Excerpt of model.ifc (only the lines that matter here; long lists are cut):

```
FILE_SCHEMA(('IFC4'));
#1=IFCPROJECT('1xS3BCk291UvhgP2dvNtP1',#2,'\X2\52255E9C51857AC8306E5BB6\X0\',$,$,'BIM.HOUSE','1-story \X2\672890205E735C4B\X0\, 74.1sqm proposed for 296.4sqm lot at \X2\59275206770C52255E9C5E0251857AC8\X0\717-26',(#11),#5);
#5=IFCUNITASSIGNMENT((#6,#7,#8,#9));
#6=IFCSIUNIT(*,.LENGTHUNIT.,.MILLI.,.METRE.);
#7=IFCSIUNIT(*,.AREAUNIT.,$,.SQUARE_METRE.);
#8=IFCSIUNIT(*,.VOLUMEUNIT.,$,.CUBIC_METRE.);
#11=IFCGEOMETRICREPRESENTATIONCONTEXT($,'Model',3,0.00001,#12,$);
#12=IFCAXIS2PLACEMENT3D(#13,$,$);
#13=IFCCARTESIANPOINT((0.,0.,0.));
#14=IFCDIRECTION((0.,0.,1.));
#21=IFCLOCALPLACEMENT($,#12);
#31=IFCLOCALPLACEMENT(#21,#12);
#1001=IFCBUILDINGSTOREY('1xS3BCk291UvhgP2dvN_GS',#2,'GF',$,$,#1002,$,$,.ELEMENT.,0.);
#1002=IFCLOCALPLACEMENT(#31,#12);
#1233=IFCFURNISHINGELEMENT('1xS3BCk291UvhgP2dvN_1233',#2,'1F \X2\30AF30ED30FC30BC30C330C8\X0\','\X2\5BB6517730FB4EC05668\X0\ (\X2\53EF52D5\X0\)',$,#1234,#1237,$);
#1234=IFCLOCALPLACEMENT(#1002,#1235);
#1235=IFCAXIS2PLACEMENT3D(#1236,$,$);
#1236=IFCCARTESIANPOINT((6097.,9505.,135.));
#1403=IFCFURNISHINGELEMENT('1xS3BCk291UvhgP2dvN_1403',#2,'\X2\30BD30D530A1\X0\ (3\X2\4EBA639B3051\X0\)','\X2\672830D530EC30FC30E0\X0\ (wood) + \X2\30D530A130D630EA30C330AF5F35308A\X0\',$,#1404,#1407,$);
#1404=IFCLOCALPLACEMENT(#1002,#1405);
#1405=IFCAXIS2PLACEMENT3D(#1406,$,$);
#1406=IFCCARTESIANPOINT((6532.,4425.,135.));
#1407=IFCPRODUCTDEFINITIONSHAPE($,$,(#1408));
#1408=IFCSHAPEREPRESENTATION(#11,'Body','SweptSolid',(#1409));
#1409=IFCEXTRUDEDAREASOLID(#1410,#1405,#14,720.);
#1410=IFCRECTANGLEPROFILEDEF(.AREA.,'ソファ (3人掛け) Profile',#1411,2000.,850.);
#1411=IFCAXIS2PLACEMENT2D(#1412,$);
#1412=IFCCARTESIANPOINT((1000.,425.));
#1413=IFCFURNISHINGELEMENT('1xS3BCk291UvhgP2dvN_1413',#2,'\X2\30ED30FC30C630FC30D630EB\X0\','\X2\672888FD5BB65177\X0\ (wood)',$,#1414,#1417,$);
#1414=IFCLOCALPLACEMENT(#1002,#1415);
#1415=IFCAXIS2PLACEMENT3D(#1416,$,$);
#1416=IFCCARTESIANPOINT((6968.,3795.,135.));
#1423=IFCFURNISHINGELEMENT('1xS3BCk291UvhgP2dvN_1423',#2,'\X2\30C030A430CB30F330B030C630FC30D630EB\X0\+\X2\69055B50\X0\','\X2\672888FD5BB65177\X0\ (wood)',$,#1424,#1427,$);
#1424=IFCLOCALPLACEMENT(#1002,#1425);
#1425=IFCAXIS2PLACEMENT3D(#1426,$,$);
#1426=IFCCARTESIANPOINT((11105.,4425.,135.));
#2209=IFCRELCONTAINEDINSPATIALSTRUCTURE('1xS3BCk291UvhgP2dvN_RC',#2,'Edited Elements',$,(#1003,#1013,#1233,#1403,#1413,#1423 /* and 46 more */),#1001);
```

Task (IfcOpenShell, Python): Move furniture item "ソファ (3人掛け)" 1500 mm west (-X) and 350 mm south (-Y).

```python
import ifcopenshell
import ifcopenshell.api.geometry
import ifcopenshell.util.placement

model = ifcopenshell.open("model.ifc")

item = model.by_guid("1xS3BCk291UvhgP2dvN_1403")
matrix = ifcopenshell.util.placement.get_local_placement(item.ObjectPlacement)
matrix[0, 3] -= 1500.0
matrix[1, 3] -= 350.0
ifcopenshell.api.geometry.edit_object_placement(model, product=item, matrix=matrix, is_si=False)

print(ifcopenshell.util.placement.get_local_placement(item.ObjectPlacement).round(3) + 0.0)

model.write("model-out.ifc")
```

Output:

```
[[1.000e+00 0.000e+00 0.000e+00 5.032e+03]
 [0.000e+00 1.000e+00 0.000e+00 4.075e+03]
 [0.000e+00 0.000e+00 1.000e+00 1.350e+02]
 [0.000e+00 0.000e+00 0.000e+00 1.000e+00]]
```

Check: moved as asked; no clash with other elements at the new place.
